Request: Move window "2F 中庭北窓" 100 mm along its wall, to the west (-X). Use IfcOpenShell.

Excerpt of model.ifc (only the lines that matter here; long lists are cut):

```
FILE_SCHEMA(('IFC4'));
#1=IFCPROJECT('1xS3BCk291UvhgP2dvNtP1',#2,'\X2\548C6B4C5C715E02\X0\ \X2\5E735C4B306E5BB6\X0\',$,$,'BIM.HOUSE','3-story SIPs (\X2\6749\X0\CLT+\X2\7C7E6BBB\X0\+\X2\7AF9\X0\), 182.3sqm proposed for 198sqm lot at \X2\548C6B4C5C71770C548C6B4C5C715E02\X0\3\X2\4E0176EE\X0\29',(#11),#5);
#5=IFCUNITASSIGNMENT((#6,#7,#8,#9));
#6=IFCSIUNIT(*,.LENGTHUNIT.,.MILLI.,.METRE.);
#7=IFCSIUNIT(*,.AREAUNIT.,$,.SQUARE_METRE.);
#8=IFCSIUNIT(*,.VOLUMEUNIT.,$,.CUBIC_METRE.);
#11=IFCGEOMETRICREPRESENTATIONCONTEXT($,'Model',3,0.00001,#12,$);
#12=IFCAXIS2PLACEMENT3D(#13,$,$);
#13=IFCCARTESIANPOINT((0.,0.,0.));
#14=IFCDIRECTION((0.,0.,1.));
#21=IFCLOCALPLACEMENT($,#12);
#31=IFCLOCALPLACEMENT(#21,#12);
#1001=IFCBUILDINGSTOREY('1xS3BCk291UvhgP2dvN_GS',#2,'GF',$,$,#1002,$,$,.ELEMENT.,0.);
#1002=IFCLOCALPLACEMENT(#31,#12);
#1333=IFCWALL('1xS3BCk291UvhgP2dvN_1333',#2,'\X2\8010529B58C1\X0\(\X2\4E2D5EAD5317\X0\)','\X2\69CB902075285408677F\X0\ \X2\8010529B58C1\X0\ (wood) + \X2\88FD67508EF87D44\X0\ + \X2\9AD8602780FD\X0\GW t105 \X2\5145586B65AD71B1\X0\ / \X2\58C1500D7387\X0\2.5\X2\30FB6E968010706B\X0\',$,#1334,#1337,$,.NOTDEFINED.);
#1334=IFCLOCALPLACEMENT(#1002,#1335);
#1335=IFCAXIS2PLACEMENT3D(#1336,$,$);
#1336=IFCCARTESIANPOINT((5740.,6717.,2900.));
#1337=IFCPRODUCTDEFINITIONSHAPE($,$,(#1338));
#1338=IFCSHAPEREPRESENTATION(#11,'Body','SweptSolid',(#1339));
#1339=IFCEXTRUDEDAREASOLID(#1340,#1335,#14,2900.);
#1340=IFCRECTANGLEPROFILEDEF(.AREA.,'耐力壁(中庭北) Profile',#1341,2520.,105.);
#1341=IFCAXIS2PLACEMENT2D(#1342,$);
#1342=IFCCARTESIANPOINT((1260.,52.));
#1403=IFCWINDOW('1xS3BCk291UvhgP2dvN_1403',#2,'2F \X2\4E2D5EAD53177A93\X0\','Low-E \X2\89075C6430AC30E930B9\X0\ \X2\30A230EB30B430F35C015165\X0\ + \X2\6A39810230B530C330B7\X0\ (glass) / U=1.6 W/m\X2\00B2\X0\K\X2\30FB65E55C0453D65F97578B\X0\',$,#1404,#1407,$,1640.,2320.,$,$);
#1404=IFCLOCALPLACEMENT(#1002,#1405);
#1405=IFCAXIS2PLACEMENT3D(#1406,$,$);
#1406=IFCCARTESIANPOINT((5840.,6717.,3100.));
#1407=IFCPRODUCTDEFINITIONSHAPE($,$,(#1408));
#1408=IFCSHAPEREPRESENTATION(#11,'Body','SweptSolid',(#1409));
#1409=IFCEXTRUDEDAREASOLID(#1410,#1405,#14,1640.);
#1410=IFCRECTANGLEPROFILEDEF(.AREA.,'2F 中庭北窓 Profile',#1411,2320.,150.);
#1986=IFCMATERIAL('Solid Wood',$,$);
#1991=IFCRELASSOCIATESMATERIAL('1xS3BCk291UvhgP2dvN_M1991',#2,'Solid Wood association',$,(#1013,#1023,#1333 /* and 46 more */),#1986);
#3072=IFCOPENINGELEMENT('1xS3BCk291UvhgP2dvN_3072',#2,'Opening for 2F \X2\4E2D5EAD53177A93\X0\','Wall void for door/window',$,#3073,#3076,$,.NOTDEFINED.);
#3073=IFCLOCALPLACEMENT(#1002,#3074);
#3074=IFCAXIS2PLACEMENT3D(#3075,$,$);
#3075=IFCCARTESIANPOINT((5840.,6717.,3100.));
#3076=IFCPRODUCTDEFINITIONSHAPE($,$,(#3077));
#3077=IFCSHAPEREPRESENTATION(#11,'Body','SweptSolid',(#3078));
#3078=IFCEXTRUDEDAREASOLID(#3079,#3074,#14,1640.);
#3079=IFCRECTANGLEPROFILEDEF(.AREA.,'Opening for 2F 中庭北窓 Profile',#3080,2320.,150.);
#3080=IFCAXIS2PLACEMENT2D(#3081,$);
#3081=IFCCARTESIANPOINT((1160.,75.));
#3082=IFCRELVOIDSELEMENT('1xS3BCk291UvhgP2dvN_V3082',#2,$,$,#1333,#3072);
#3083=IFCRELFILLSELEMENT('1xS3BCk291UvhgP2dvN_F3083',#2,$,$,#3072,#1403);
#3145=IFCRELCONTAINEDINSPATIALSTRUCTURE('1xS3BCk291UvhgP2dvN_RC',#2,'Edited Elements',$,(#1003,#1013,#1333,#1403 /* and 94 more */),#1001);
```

```python
import ifcopenshell
import ifcopenshell.api.geometry
import ifcopenshell.util.placement
import ifcopenshell.util.unit

model = ifcopenshell.open("model.ifc")
unit_scale = ifcopenshell.util.unit.calculate_unit_scale(model)

window = model.by_guid("1xS3BCk291UvhgP2dvN_1403")
opening = window.FillsVoids[0].RelatingOpeningElement
wall = opening.VoidsElements[0].RelatingBuildingElement

wall_matrix = ifcopenshell.util.placement.get_local_placement(wall.ObjectPlacement)
shift = wall_matrix[:3, 0] * -0.1 / unit_scale
before = ifcopenshell.util.placement.get_local_placement(window.ObjectPlacement)[:3, 3].copy()

# The window is not placed relative to its opening, so move both.
for product in (opening, window):
    matrix = ifcopenshell.util.placement.get_local_placement(product.ObjectPlacement)
    matrix[:3, 3] += shift
    ifcopenshell.api.geometry.edit_object_placement(model, product=product, matrix=matrix, is_si=False)

after = ifcopenshell.util.placement.get_local_placement(window.ObjectPlacement)[:3, 3]
print("window moved by", (after - before).round(3) + 0.0)

model.write("model_rev.ifc")
```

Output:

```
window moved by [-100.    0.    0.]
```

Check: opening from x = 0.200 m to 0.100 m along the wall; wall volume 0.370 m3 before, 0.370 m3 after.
